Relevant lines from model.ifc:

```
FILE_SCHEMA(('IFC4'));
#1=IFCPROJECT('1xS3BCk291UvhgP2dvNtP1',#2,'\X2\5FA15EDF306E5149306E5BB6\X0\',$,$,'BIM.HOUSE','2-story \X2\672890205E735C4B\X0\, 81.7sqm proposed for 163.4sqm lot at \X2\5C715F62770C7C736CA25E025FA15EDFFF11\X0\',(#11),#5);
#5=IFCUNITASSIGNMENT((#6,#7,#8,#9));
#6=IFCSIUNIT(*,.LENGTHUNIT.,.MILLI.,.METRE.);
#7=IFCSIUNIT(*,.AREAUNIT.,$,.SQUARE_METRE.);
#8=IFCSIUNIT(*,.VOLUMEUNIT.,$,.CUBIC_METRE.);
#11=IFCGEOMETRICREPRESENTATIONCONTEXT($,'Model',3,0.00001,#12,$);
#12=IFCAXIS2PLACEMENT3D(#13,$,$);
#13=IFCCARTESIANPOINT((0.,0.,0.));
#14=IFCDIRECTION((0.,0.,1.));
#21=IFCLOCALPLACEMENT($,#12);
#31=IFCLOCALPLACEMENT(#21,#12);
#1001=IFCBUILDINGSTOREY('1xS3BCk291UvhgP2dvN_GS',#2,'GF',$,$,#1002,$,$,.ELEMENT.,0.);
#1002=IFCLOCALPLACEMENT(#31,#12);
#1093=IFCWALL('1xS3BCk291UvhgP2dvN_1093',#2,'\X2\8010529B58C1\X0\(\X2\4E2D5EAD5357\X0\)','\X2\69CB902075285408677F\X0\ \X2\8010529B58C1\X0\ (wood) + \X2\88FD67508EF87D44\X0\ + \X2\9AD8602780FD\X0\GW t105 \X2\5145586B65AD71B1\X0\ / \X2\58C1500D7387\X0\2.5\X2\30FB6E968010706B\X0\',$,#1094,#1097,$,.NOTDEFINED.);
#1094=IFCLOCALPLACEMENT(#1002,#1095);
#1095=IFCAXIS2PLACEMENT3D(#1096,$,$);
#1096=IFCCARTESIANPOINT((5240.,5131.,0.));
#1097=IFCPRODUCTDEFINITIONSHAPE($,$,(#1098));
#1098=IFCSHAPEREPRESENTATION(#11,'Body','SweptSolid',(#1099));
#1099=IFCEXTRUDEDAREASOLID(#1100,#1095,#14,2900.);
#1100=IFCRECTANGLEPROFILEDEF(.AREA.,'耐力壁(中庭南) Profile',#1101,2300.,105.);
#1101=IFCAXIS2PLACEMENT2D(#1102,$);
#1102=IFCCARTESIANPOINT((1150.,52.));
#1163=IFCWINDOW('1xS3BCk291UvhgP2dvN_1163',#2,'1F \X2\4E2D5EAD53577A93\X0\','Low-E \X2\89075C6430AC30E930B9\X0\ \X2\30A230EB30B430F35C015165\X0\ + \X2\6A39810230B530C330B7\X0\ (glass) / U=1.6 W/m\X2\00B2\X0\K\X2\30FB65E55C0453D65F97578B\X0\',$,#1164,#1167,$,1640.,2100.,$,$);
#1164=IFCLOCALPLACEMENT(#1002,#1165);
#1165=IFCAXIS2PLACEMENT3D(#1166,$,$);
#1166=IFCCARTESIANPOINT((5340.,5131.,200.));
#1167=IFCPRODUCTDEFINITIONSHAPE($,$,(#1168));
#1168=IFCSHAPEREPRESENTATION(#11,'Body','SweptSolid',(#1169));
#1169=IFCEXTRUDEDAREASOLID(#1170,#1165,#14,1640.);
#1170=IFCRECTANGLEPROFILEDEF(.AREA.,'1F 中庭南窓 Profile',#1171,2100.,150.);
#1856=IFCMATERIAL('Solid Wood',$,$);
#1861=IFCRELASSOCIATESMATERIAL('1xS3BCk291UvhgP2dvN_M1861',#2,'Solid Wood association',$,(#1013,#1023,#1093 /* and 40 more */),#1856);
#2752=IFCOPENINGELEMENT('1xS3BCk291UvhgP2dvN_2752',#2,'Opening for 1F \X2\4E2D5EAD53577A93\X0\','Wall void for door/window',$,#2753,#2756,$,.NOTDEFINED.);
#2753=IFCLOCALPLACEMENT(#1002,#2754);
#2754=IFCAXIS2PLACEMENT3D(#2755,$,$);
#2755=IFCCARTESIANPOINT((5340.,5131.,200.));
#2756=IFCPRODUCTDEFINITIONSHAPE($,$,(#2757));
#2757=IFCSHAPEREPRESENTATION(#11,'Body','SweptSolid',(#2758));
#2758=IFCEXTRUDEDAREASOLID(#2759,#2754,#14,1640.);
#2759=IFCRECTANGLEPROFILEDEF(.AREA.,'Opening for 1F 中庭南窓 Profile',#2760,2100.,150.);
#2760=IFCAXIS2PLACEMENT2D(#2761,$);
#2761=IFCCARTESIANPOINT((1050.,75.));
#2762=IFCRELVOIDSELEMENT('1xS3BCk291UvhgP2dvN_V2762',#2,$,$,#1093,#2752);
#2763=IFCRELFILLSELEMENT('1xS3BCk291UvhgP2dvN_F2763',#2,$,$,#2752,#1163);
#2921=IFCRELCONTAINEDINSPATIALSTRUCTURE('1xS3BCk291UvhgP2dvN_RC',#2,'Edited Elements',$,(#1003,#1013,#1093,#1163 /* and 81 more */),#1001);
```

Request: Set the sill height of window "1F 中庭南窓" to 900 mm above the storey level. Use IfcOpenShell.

```python
import numpy as np
import ifcopenshell
import ifcopenshell.api.geometry
import ifcopenshell.geom
import ifcopenshell.util.element
import ifcopenshell.util.placement
import ifcopenshell.util.shape
import ifcopenshell.util.unit

model = ifcopenshell.open("model.ifc")
unit_scale = ifcopenshell.util.unit.calculate_unit_scale(model)

window = model.by_guid("1xS3BCk291UvhgP2dvN_1163")
opening = window.FillsVoids[0].RelatingOpeningElement
storey = ifcopenshell.util.element.get_container(window, ifc_class="IfcBuildingStorey")
level = ifcopenshell.util.placement.get_local_placement(storey.ObjectPlacement)[2, 3]

# The opening's origin need not be at the sill, so measure its lowest point.
shape = ifcopenshell.geom.create_shape(ifcopenshell.geom.settings(), opening)
bottom = ifcopenshell.util.shape.get_shape_bottom_elevation(shape, shape.geometry) / unit_scale
dz = level + 900.0 - bottom

shift = np.array([0.0, 0.0, dz])
# The window is not placed relative to its opening, so move both.
for product in (opening, window):
    matrix = ifcopenshell.util.placement.get_local_placement(product.ObjectPlacement)
    matrix[:3, 3] += shift
    ifcopenshell.api.geometry.edit_object_placement(model, product=product, matrix=matrix, is_si=False)

print(f"moved by {dz * unit_scale:+.3f} m")

model.write("model_updated.ifc")
```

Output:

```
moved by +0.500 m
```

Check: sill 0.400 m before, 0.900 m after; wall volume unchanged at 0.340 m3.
